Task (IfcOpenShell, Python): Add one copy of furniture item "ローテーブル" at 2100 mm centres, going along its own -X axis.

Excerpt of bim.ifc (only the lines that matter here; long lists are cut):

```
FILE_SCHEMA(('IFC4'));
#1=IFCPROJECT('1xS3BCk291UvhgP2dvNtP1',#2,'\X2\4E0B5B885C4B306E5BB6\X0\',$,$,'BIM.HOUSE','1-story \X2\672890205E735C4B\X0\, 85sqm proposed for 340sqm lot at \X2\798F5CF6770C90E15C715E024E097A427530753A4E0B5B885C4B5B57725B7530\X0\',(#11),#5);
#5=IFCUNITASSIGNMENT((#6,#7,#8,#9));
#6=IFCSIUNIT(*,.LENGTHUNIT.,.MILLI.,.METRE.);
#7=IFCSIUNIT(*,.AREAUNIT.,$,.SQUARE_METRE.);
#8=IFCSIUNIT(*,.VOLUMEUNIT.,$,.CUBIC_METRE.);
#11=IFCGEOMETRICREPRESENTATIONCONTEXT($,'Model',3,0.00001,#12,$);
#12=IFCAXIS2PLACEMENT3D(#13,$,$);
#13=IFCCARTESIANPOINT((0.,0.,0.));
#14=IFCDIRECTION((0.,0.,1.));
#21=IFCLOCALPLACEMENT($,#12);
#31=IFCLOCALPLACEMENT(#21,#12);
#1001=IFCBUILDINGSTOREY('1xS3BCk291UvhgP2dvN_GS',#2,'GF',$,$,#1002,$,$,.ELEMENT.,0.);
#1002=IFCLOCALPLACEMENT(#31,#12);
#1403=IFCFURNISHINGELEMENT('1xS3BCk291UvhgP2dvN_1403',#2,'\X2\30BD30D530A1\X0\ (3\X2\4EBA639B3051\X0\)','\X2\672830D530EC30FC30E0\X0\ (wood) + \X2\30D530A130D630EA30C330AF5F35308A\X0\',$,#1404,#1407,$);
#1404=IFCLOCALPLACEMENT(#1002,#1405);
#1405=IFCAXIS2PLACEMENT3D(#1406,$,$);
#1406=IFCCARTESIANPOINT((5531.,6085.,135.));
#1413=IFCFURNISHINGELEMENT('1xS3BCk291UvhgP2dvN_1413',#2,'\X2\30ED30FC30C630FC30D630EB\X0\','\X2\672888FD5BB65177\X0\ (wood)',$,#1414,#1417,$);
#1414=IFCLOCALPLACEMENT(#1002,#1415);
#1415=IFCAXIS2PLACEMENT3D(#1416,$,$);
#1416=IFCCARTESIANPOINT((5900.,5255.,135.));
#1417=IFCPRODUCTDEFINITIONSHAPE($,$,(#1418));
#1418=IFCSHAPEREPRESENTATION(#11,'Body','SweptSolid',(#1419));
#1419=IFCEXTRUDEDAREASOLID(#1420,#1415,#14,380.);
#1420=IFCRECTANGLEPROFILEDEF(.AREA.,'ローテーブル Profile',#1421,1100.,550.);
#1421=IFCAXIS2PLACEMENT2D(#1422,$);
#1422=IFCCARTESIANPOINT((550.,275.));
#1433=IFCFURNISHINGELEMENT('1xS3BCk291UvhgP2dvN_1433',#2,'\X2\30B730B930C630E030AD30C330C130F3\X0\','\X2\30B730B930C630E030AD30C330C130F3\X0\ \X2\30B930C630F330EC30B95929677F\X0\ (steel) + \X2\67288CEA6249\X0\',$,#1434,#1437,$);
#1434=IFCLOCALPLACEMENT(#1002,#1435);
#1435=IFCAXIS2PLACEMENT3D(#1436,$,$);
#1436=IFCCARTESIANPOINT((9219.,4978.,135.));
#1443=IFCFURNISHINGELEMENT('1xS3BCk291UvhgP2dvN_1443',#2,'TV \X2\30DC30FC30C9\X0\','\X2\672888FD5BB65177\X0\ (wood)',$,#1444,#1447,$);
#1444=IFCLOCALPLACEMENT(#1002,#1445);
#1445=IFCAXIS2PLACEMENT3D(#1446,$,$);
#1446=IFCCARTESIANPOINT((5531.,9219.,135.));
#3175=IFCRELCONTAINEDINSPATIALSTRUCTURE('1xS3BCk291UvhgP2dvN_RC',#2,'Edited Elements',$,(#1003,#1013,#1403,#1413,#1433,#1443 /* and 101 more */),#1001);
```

```python
import ifcopenshell
import ifcopenshell.api.geometry
import ifcopenshell.api.root
import ifcopenshell.util.element
import ifcopenshell.util.placement
import ifcopenshell.util.unit

model = ifcopenshell.open("bim.ifc")
unit_scale = ifcopenshell.util.unit.calculate_unit_scale(model)


def reuse_history(source, copy):
    """copy_class also copies each property set's owner history, people and application; keep the originals."""
    for rel in copy.IsDefinedBy:
        if rel.is_a("IfcRelDefinesByProperties") and (history := rel.RelatingPropertyDefinition.OwnerHistory):
            rel.RelatingPropertyDefinition.OwnerHistory = source.OwnerHistory
            ifcopenshell.util.element.remove_deep2(model, history)


source = model.by_guid("1xS3BCk291UvhgP2dvN_1413")
base = ifcopenshell.util.placement.get_local_placement(source.ObjectPlacement)
step = -base[:3, 0] * 2.1 / unit_scale

for i in range(1, 2):
    copy = ifcopenshell.api.root.copy_class(model, product=source)
    copy.Representation = ifcopenshell.util.element.copy_deep(
        model, source.Representation, exclude=["IfcGeometricRepresentationContext", "IfcRepresentationMap"]
    )
    reuse_history(source, copy)
    matrix = base.copy()
    matrix[:3, 3] += i * step
    print("added at", matrix[:3, 3].round(3) + 0.0)
    ifcopenshell.api.geometry.edit_object_placement(model, product=copy, matrix=matrix, is_si=False)

model.write("bim_edited.ifc")
```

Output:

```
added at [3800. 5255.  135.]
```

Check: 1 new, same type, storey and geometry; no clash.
